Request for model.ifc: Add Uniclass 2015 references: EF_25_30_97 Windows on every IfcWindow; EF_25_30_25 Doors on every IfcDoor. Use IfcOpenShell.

First a look at what the model holds.

```python
import ifcopenshell

model = ifcopenshell.open("model.ifc")
print(model.schema)
print("classifications:", [c.Name for c in model.by_type("IfcClassification")])
for ifc_class in ("IfcDoor", "IfcRoof", "IfcStair", "IfcWall", "IfcWindow"):
    print(ifc_class, len(model.by_type(ifc_class)))
```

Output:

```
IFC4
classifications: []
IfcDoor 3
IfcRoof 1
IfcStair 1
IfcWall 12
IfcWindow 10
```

```python
import ifcopenshell
import ifcopenshell.api.classification

model = ifcopenshell.open("model.ifc")

system = ifcopenshell.api.classification.add_classification(model, classification="Uniclass 2015")

codes = {
    "IfcWindow": ("EF_25_30_97", "Windows"),
    "IfcDoor": ("EF_25_30_25", "Doors"),
}
for ifc_class, (code, name) in codes.items():
    products = model.by_type(ifc_class)
    ifcopenshell.api.classification.add_reference(
        model, products=products, classification=system, identification=code, name=name
    )
    print(code, len(products))

model.write("model_updated.ifc")
```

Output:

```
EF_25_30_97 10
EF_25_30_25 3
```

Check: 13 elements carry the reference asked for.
